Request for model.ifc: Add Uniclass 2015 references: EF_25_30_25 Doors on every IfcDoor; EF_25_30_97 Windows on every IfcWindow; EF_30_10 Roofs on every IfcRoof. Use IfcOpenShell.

First a look at what the model holds.

```python
import ifcopenshell

model = ifcopenshell.open("model.ifc")
print(model.schema)
print("classifications:", [c.Name for c in model.by_type("IfcClassification")])
for ifc_class in ("IfcDoor", "IfcRoof", "IfcStair", "IfcWall", "IfcWindow"):
    print(ifc_class, len(model.by_type(ifc_class)))
```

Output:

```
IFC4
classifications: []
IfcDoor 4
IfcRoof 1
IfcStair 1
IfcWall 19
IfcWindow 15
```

```python
import ifcopenshell
import ifcopenshell.api.classification

model = ifcopenshell.open("model.ifc")

system = ifcopenshell.api.classification.add_classification(model, classification="Uniclass 2015")

codes = {
    "IfcDoor": ("EF_25_30_25", "Doors"),
    "IfcWindow": ("EF_25_30_97", "Windows"),
    "IfcRoof": ("EF_30_10", "Roofs"),
}
for ifc_class, (code, name) in codes.items():
    products = model.by_type(ifc_class)
    ifcopenshell.api.classification.add_reference(
        model, products=products, classification=system, identification=code, name=name
    )
    print(code, len(products))

model.write("model-out.ifc")
```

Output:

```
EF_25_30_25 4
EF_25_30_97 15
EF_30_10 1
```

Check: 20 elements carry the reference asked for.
